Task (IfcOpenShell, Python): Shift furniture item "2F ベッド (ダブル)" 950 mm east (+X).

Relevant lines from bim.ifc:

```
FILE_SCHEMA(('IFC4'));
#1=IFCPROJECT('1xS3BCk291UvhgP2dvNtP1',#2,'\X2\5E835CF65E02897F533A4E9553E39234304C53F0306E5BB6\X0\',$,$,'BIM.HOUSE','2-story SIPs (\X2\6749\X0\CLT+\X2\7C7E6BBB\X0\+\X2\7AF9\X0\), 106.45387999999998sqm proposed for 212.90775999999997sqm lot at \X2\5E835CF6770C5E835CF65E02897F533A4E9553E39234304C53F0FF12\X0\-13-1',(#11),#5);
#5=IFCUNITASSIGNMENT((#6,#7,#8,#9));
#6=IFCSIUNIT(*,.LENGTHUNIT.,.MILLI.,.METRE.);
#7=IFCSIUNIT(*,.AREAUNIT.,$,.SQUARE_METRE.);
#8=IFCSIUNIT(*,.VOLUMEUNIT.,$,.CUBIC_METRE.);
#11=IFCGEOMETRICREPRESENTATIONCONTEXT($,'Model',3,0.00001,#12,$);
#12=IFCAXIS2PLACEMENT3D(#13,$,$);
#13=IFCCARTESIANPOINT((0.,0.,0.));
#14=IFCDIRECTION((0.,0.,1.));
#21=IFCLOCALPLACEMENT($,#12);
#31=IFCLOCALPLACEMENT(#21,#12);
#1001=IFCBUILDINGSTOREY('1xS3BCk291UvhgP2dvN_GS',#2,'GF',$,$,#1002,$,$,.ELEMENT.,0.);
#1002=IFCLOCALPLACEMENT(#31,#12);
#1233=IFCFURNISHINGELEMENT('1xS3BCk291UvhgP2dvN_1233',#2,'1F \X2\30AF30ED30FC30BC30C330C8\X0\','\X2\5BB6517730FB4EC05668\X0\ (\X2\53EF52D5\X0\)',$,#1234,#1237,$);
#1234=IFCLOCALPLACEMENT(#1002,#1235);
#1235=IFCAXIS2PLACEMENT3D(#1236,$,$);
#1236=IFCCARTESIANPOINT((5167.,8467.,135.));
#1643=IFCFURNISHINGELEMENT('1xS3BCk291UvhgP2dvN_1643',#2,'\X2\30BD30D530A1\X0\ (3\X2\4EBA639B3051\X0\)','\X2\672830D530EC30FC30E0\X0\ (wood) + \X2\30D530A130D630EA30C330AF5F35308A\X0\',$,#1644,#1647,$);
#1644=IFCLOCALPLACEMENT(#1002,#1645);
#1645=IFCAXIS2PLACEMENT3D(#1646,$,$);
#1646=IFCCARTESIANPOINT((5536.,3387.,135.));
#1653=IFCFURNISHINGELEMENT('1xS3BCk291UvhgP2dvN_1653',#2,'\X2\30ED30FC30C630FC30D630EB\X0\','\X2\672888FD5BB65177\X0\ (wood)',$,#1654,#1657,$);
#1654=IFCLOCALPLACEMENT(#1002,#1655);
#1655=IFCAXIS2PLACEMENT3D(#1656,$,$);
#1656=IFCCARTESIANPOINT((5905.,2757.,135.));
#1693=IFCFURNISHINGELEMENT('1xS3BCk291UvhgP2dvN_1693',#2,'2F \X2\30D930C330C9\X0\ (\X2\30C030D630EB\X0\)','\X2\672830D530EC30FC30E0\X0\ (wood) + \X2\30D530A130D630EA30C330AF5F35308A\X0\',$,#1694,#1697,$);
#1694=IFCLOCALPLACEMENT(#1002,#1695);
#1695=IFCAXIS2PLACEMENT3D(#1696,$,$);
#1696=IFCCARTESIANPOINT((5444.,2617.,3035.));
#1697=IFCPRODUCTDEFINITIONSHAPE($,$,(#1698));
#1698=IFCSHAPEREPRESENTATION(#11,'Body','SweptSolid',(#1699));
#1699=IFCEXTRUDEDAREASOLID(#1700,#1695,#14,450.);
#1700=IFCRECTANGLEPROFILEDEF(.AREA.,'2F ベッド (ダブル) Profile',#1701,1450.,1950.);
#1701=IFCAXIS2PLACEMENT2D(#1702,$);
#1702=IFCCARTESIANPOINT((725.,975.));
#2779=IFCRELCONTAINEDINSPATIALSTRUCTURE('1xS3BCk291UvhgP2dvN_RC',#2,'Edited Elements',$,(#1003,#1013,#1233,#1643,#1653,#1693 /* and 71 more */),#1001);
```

```python
import ifcopenshell
import ifcopenshell.api.geometry
import ifcopenshell.util.placement

model = ifcopenshell.open("bim.ifc")

item = model.by_guid("1xS3BCk291UvhgP2dvN_1693")
matrix = ifcopenshell.util.placement.get_local_placement(item.ObjectPlacement)
matrix[0, 3] += 950.0
ifcopenshell.api.geometry.edit_object_placement(model, product=item, matrix=matrix, is_si=False)

print(ifcopenshell.util.placement.get_local_placement(item.ObjectPlacement).round(3) + 0.0)

model.write("bim_v2.ifc")
```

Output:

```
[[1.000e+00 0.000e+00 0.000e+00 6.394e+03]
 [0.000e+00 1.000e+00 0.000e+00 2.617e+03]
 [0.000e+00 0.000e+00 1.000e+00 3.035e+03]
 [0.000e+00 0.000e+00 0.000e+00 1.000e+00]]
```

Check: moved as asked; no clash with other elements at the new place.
